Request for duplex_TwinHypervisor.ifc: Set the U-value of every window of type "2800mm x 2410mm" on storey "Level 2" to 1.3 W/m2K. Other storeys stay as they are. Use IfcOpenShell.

First a look at what the model holds.

```python
import ifcopenshell
import ifcopenshell.util.element

model = ifcopenshell.open("duplex_TwinHypervisor.ifc")
print(model.schema)
storey = next(s for s in model.by_type("IfcBuildingStorey") if s.Name == "Level 2")
windows = [e for e in ifcopenshell.util.element.get_decomposition(storey) if e.is_a("IfcWindow")]
seen = {}
for e in windows:
    element_type = ifcopenshell.util.element.get_type(e)
    key = (element_type.Name if element_type != e and element_type else None, ifcopenshell.util.element.get_pset(e, "Pset_WindowCommon", "ThermalTransmittance"))
    seen[key] = seen.get(key, 0) + 1
for (name, value), count in sorted(seen.items(), key=str):
    print(count, "x", name, "|", value)
```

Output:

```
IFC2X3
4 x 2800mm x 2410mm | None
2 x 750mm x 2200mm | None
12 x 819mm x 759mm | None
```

```python
import ifcopenshell
import ifcopenshell.api.pset
import ifcopenshell.util.element

model = ifcopenshell.open("duplex_TwinHypervisor.ifc")

storey = next(s for s in model.by_type("IfcBuildingStorey") if s.Name == "Level 2")
windows = [e for e in ifcopenshell.util.element.get_decomposition(storey) if e.is_a("IfcWindow")]

count = 0
for e in windows:
    element_type = ifcopenshell.util.element.get_type(e)
    if element_type in (None, e) or element_type.Name != "2800mm x 2410mm":
        continue
    # add_pset returns the element's existing set when there is one.
    pset = ifcopenshell.api.pset.add_pset(model, product=e, name="Pset_WindowCommon")
    ifcopenshell.api.pset.edit_pset(model, pset=pset, properties={"ThermalTransmittance": 1.3})
    count += 1

print(count, "windows updated")

model.write("duplex_TwinHypervisor_updated.ifc")
```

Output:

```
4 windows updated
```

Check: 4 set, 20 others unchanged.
